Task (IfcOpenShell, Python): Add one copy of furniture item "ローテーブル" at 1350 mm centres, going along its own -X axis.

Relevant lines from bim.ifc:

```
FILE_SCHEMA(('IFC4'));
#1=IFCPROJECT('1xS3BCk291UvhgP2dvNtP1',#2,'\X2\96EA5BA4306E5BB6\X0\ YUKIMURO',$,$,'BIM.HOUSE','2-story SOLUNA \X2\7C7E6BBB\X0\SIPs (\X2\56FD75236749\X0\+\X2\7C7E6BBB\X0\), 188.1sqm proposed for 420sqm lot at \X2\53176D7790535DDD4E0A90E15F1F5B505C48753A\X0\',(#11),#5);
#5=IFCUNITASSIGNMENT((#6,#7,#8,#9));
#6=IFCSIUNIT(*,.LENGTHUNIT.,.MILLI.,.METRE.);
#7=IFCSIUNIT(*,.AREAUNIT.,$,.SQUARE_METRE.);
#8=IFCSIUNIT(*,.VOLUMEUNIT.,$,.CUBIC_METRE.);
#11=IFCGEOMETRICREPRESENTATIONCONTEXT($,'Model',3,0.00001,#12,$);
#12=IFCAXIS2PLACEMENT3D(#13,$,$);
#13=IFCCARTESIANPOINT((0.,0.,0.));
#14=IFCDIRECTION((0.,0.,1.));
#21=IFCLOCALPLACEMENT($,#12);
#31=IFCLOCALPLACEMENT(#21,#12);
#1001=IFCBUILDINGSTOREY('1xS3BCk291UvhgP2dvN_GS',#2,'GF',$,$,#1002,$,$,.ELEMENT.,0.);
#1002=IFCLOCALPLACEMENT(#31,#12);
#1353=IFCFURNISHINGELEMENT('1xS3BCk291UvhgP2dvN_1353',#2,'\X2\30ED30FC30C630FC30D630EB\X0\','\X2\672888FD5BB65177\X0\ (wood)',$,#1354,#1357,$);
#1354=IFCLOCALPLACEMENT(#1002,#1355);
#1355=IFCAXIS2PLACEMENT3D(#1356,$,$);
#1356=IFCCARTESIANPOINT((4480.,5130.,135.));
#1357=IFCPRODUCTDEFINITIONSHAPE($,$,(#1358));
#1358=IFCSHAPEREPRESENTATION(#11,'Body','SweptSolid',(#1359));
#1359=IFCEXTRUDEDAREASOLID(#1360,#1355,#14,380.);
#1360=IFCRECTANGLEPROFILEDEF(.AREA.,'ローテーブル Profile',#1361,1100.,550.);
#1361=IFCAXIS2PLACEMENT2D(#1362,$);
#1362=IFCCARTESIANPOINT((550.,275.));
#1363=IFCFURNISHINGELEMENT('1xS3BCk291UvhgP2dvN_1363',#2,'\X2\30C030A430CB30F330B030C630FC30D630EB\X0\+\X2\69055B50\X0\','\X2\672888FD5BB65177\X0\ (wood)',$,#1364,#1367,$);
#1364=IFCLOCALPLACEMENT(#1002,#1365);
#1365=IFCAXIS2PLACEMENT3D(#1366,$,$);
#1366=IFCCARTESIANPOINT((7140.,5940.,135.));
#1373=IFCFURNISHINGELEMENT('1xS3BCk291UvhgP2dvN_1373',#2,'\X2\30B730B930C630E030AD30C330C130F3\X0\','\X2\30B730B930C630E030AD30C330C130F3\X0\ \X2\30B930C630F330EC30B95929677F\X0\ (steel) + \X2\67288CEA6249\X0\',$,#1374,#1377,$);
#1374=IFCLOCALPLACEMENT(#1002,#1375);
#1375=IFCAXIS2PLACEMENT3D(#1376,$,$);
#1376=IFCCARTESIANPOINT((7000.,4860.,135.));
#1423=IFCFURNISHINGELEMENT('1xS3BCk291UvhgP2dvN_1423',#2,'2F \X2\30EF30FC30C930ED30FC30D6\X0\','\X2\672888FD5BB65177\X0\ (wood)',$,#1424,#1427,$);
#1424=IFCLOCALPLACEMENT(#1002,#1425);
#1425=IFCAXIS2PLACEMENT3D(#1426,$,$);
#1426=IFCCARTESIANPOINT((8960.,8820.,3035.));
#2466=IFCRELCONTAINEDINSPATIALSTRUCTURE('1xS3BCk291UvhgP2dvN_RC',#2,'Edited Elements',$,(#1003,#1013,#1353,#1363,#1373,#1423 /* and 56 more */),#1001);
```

```python
import ifcopenshell
import ifcopenshell.api.geometry
import ifcopenshell.api.root
import ifcopenshell.util.element
import ifcopenshell.util.placement
import ifcopenshell.util.unit

model = ifcopenshell.open("bim.ifc")
unit_scale = ifcopenshell.util.unit.calculate_unit_scale(model)


def reuse_history(source, copy):
    """copy_class also copies each property set's owner history, people and application; keep the originals."""
    for rel in copy.IsDefinedBy:
        if rel.is_a("IfcRelDefinesByProperties") and (history := rel.RelatingPropertyDefinition.OwnerHistory):
            rel.RelatingPropertyDefinition.OwnerHistory = source.OwnerHistory
            ifcopenshell.util.element.remove_deep2(model, history)


source = model.by_id(1353)
base = ifcopenshell.util.placement.get_local_placement(source.ObjectPlacement)
step = -base[:3, 0] * 1.35 / unit_scale

for i in range(1, 2):
    copy = ifcopenshell.api.root.copy_class(model, product=source)
    copy.Representation = ifcopenshell.util.element.copy_deep(
        model, source.Representation, exclude=["IfcGeometricRepresentationContext", "IfcRepresentationMap"]
    )
    reuse_history(source, copy)
    matrix = base.copy()
    matrix[:3, 3] += i * step
    print("added at", matrix[:3, 3].round(3) + 0.0)
    ifcopenshell.api.geometry.edit_object_placement(model, product=copy, matrix=matrix, is_si=False)

model.write("bim-out.ifc")
```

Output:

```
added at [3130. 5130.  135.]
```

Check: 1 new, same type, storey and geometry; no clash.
